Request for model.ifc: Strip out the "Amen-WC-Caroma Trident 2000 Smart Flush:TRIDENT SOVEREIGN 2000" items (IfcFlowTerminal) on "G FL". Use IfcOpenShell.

First a look at what the model holds.

```python
import ifcopenshell
import ifcopenshell.util.element

model = ifcopenshell.open("model.ifc")
print(model.schema)
storey = next(s for s in model.by_type("IfcBuildingStorey") if s.Name == "G FL")
terminals = [e for e in ifcopenshell.util.element.get_decomposition(storey) if e.is_a("IfcFlowTerminal")]
seen = {}
for e in terminals:
    element_type = ifcopenshell.util.element.get_type(e)
    name = element_type.Name if element_type not in (None, e) else None
    seen[name] = seen.get(name, 0) + 1
for name, count in sorted(seen.items(), key=str):
    print(count, "x", name)
```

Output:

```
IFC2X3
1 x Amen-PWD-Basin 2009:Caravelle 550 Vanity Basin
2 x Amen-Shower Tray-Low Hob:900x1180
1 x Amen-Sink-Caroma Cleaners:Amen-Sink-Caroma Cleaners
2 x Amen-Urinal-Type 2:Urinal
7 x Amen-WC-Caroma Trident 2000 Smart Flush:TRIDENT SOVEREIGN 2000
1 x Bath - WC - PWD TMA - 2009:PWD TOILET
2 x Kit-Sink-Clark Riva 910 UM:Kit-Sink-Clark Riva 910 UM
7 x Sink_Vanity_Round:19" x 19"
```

```python
import ifcopenshell
import ifcopenshell.api.root
import ifcopenshell.util.element

model = ifcopenshell.open("model.ifc")

storey = next(s for s in model.by_type("IfcBuildingStorey") if s.Name == "G FL")
terminals = [e for e in ifcopenshell.util.element.get_decomposition(storey) if e.is_a("IfcFlowTerminal")]
targets = [e for e in terminals if (t := ifcopenshell.util.element.get_type(e)) not in (None, e) and t.Name == "Amen-WC-Caroma Trident 2000 Smart Flush:TRIDENT SOVEREIGN 2000"]

for e in targets:
    ifcopenshell.api.root.remove_product(model, product=e)
print(len(targets), "removed")

model.write("model_rev.ifc")
```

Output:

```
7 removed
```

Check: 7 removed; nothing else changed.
